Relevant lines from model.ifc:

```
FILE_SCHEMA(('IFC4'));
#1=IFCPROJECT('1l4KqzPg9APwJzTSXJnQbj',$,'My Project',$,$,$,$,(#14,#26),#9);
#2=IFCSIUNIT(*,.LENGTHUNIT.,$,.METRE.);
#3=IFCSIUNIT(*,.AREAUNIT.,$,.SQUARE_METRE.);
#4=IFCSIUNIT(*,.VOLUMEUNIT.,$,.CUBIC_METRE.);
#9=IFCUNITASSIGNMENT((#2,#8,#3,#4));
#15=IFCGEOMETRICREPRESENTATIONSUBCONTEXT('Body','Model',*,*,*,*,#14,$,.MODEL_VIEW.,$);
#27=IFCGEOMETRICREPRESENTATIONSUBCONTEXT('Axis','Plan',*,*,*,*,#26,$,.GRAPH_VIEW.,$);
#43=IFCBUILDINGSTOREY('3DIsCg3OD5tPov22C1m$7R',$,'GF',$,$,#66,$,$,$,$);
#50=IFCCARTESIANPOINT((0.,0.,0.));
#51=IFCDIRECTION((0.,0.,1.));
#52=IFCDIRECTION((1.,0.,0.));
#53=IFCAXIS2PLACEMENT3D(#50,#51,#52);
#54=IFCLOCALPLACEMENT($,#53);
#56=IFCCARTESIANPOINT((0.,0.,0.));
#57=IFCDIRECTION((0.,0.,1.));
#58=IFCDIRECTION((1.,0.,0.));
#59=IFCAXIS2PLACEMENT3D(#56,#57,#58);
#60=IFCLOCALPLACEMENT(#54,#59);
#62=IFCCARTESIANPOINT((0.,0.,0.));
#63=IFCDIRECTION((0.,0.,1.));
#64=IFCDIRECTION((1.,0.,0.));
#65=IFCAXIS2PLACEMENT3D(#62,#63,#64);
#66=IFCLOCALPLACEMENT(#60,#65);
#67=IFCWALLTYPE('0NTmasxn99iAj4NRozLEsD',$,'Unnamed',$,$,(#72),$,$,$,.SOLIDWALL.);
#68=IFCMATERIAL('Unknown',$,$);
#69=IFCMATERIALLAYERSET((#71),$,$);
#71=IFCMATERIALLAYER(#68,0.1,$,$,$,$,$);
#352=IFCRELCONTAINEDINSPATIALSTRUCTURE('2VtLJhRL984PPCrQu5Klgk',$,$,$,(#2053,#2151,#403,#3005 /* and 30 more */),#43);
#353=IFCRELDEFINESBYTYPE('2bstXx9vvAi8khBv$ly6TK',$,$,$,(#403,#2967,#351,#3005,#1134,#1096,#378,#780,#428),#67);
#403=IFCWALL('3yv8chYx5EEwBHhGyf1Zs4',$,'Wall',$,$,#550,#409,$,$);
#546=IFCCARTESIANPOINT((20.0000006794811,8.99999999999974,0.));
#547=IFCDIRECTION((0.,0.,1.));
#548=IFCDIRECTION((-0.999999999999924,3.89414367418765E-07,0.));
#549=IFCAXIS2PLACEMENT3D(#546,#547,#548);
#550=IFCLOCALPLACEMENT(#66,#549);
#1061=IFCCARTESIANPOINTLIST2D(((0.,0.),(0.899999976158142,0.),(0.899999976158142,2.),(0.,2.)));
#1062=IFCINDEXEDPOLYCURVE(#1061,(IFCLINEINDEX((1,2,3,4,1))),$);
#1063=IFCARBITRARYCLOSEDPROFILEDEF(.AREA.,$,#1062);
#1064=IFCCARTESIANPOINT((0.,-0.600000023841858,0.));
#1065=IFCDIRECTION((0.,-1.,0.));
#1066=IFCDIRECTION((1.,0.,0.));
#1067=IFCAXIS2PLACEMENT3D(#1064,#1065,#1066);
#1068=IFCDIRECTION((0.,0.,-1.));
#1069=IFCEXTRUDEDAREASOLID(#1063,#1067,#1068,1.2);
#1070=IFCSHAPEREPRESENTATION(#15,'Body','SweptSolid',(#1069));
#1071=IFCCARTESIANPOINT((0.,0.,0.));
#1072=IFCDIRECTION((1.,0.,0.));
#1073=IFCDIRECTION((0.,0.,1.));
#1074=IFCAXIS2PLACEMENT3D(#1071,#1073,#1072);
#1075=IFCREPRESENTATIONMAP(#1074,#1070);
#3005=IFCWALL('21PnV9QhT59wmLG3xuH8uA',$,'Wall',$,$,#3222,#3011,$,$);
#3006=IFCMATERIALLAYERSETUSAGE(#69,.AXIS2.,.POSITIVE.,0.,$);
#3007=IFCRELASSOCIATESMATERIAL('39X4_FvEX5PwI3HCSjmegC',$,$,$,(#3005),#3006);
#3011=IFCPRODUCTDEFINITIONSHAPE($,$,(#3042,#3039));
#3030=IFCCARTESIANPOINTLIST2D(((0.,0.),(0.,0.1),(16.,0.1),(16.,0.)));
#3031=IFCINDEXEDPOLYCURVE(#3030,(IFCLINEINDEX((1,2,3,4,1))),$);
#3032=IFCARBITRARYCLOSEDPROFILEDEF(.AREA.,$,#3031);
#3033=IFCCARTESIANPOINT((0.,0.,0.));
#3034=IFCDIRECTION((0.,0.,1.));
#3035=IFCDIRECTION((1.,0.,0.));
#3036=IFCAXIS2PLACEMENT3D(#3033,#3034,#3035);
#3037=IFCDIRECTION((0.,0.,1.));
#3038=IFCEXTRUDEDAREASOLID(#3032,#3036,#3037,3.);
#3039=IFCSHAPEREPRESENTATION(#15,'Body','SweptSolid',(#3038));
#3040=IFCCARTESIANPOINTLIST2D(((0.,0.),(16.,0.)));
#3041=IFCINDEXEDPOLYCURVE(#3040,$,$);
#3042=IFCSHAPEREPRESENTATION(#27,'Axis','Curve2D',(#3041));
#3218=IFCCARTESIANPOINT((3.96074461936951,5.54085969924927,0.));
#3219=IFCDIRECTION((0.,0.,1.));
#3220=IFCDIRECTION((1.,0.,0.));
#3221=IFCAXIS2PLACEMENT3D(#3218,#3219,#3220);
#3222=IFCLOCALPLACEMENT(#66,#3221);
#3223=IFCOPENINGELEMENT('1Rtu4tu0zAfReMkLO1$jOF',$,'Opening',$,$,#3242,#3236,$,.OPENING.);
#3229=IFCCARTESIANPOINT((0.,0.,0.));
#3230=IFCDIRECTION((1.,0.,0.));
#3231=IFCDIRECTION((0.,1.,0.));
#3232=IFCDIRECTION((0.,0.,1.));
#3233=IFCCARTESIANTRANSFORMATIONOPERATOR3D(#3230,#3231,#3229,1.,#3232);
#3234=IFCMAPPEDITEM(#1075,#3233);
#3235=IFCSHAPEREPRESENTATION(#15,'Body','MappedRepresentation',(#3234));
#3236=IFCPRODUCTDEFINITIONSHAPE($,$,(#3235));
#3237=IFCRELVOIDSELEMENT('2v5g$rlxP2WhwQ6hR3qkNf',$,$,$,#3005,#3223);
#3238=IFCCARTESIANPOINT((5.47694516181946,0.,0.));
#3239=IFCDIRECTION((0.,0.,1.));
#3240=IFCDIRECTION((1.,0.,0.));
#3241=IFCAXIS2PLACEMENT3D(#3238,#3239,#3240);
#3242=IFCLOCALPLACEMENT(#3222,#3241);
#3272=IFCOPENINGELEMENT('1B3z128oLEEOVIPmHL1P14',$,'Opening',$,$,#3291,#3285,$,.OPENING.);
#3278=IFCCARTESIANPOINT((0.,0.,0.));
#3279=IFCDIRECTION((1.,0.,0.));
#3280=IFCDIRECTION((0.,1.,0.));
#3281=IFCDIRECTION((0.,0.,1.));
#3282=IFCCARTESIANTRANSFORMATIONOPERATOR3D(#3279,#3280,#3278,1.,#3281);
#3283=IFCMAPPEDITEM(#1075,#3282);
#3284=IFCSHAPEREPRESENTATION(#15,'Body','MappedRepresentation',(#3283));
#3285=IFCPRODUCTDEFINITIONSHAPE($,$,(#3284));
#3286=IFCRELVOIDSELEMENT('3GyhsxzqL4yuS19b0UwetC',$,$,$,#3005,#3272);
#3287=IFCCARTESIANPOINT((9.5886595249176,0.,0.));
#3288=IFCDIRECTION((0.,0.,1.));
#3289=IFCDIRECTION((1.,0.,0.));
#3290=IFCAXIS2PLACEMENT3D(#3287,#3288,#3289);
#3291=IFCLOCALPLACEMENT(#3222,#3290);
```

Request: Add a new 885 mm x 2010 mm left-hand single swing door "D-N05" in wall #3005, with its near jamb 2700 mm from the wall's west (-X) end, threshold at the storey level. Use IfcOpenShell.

```python
import numpy as np
import ifcopenshell
import ifcopenshell.api.feature
import ifcopenshell.api.geometry
import ifcopenshell.api.root
import ifcopenshell.api.spatial
import ifcopenshell.geom
import ifcopenshell.util.element
import ifcopenshell.util.placement
import ifcopenshell.util.representation
import ifcopenshell.util.shape
import ifcopenshell.util.unit

model = ifcopenshell.open("model.ifc")
unit_scale = ifcopenshell.util.unit.calculate_unit_scale(model)
settings = ifcopenshell.geom.settings()


def volume(element):
    """Net volume in cubic metres, openings subtracted."""
    shape = ifcopenshell.geom.create_shape(settings, element)
    return ifcopenshell.util.shape.get_volume(shape.geometry)


wall = model.by_guid("21PnV9QhT59wmLG3xuH8uA")
storey = ifcopenshell.util.element.get_container(wall, ifc_class="IfcBuildingStorey")
context = ifcopenshell.util.representation.get_context(model, "Model", "Body", "MODEL_VIEW")
before = volume(wall)

width, height, from_end, sill = 0.885, 2.01, 2.7, 0.0  # metres

# The wall runs along its own X axis, and the end named is its -X end.
wall_shape = ifcopenshell.geom.create_shape(settings, wall)
x, y, z = ifcopenshell.util.shape.get_vertices(wall_shape.geometry).T
start = x.min() + from_end
face, thickness = float(y.min()), float(y.max() - y.min())
wall_matrix = ifcopenshell.util.placement.get_local_placement(wall.ObjectPlacement)
level = ifcopenshell.util.placement.get_local_placement(storey.ObjectPlacement)[2, 3]


def in_wall(x, y):
    """Placement at x, y metres in the wall's axes, at sill height."""
    matrix = wall_matrix.copy()
    matrix[:, 3] = wall_matrix @ np.array([x / unit_scale, y / unit_scale, 0.0, 1.0])
    matrix[2, 3] = level + sill / unit_scale
    return matrix


# Opening: a box that overshoots both wall faces by 50 mm.
opening = ifcopenshell.api.root.create_entity(model, ifc_class="IfcOpeningElement", predefined_type="OPENING")
box = ifcopenshell.api.geometry.add_wall_representation(
    model, context=context, length=width, height=height, thickness=thickness + 0.1
)
ifcopenshell.api.geometry.assign_representation(model, product=opening, representation=box)
ifcopenshell.api.geometry.edit_object_placement(model, product=opening, matrix=in_wall(start, face - 0.05), is_si=False)
ifcopenshell.api.feature.add_feature(model, feature=opening, element=wall)

door = ifcopenshell.api.root.create_entity(model, ifc_class="IfcDoor", name="D-N05", predefined_type="DOOR")
door.OverallWidth, door.OverallHeight = width / unit_scale, height / unit_scale
door.OperationType = "SINGLE_SWING_LEFT"
body = ifcopenshell.api.geometry.add_door_representation(
    model,
    context=context,
    overall_width=door.OverallWidth,
    overall_height=door.OverallHeight,
    operation_type="SINGLE_SWING_LEFT",
    lining_properties={"LiningDepth": thickness / unit_scale, "ThresholdDepth": thickness / unit_scale},
)
ifcopenshell.api.geometry.assign_representation(model, product=door, representation=body)
ifcopenshell.api.spatial.assign_container(model, products=[door], relating_structure=storey)
ifcopenshell.api.feature.add_filling(model, opening=opening, element=door)

# The lining spans the wall, so the door starts at the wall face.
ifcopenshell.api.geometry.edit_object_placement(model, product=door, matrix=in_wall(start, face), is_si=False)

after = volume(wall)

print(f"wall volume {before:.3f} -> {after:.3f} m3")

model.write("model-out.ifc")
```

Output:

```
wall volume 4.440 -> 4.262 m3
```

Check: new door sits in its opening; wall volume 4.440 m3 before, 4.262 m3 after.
